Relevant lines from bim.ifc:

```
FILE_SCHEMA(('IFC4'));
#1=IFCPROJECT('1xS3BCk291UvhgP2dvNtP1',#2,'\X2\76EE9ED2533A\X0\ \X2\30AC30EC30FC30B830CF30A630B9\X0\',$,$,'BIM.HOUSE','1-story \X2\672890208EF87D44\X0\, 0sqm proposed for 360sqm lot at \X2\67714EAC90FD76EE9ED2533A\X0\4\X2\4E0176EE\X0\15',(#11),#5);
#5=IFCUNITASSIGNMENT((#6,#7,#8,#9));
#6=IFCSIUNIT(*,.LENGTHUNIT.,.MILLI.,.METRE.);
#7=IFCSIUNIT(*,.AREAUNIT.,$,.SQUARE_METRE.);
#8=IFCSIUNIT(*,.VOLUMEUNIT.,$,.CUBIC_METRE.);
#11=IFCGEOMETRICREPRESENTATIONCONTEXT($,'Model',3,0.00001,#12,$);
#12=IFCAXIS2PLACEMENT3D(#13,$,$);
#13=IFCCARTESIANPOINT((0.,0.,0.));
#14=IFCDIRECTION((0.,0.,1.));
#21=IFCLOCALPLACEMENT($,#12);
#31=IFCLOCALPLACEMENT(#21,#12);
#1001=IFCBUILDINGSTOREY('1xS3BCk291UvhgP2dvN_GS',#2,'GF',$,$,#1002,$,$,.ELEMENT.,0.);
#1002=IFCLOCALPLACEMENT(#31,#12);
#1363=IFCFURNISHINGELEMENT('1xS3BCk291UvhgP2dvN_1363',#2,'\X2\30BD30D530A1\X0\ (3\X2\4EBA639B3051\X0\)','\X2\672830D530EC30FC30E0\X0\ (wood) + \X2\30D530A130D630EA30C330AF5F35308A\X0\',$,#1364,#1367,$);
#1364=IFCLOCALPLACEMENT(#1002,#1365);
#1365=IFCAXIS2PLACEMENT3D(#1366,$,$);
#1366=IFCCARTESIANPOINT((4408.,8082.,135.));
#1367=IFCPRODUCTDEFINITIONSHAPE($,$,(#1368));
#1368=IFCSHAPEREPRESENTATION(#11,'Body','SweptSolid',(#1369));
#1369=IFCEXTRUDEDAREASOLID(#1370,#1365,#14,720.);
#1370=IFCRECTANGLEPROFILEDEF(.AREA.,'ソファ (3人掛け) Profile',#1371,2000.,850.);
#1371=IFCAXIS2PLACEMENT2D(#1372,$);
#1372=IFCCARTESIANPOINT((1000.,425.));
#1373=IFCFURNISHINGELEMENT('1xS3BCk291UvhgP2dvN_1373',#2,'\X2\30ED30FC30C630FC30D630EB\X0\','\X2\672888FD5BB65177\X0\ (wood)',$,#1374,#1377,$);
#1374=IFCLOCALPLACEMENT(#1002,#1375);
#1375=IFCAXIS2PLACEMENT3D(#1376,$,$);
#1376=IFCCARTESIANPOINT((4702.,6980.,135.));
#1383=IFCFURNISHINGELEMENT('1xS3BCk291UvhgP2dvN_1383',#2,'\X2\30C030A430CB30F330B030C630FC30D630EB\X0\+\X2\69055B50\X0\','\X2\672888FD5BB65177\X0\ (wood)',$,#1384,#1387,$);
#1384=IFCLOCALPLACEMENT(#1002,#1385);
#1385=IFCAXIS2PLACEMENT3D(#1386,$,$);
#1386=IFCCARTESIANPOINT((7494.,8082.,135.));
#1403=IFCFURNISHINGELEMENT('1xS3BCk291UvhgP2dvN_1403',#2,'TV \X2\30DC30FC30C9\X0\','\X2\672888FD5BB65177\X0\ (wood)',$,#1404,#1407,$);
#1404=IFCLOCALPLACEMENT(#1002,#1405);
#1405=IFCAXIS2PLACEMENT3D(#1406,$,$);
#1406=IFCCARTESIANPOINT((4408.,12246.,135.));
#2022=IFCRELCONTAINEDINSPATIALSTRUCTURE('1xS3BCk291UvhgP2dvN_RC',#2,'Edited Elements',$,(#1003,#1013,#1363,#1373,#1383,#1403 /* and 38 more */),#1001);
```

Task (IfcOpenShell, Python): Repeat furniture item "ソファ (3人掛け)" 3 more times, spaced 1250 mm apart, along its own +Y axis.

```python
import ifcopenshell
import ifcopenshell.api.geometry
import ifcopenshell.api.root
import ifcopenshell.util.element
import ifcopenshell.util.placement
import ifcopenshell.util.unit

model = ifcopenshell.open("bim.ifc")
unit_scale = ifcopenshell.util.unit.calculate_unit_scale(model)


def reuse_history(source, copy):
    """copy_class also copies each property set's owner history, people and application; keep the originals."""
    for rel in copy.IsDefinedBy:
        if rel.is_a("IfcRelDefinesByProperties") and (history := rel.RelatingPropertyDefinition.OwnerHistory):
            rel.RelatingPropertyDefinition.OwnerHistory = source.OwnerHistory
            ifcopenshell.util.element.remove_deep2(model, history)


source = model.by_guid("1xS3BCk291UvhgP2dvN_1363")
base = ifcopenshell.util.placement.get_local_placement(source.ObjectPlacement)
step = base[:3, 1] * 1.25 / unit_scale

for i in range(1, 4):
    copy = ifcopenshell.api.root.copy_class(model, product=source)
    copy.Representation = ifcopenshell.util.element.copy_deep(
        model, source.Representation, exclude=["IfcGeometricRepresentationContext", "IfcRepresentationMap"]
    )
    reuse_history(source, copy)
    matrix = base.copy()
    matrix[:3, 3] += i * step
    print("added at", matrix[:3, 3].round(3) + 0.0)
    ifcopenshell.api.geometry.edit_object_placement(model, product=copy, matrix=matrix, is_si=False)

model.write("bim_edited.ifc")
```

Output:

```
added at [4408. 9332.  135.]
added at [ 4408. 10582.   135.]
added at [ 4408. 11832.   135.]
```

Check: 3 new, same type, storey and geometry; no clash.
